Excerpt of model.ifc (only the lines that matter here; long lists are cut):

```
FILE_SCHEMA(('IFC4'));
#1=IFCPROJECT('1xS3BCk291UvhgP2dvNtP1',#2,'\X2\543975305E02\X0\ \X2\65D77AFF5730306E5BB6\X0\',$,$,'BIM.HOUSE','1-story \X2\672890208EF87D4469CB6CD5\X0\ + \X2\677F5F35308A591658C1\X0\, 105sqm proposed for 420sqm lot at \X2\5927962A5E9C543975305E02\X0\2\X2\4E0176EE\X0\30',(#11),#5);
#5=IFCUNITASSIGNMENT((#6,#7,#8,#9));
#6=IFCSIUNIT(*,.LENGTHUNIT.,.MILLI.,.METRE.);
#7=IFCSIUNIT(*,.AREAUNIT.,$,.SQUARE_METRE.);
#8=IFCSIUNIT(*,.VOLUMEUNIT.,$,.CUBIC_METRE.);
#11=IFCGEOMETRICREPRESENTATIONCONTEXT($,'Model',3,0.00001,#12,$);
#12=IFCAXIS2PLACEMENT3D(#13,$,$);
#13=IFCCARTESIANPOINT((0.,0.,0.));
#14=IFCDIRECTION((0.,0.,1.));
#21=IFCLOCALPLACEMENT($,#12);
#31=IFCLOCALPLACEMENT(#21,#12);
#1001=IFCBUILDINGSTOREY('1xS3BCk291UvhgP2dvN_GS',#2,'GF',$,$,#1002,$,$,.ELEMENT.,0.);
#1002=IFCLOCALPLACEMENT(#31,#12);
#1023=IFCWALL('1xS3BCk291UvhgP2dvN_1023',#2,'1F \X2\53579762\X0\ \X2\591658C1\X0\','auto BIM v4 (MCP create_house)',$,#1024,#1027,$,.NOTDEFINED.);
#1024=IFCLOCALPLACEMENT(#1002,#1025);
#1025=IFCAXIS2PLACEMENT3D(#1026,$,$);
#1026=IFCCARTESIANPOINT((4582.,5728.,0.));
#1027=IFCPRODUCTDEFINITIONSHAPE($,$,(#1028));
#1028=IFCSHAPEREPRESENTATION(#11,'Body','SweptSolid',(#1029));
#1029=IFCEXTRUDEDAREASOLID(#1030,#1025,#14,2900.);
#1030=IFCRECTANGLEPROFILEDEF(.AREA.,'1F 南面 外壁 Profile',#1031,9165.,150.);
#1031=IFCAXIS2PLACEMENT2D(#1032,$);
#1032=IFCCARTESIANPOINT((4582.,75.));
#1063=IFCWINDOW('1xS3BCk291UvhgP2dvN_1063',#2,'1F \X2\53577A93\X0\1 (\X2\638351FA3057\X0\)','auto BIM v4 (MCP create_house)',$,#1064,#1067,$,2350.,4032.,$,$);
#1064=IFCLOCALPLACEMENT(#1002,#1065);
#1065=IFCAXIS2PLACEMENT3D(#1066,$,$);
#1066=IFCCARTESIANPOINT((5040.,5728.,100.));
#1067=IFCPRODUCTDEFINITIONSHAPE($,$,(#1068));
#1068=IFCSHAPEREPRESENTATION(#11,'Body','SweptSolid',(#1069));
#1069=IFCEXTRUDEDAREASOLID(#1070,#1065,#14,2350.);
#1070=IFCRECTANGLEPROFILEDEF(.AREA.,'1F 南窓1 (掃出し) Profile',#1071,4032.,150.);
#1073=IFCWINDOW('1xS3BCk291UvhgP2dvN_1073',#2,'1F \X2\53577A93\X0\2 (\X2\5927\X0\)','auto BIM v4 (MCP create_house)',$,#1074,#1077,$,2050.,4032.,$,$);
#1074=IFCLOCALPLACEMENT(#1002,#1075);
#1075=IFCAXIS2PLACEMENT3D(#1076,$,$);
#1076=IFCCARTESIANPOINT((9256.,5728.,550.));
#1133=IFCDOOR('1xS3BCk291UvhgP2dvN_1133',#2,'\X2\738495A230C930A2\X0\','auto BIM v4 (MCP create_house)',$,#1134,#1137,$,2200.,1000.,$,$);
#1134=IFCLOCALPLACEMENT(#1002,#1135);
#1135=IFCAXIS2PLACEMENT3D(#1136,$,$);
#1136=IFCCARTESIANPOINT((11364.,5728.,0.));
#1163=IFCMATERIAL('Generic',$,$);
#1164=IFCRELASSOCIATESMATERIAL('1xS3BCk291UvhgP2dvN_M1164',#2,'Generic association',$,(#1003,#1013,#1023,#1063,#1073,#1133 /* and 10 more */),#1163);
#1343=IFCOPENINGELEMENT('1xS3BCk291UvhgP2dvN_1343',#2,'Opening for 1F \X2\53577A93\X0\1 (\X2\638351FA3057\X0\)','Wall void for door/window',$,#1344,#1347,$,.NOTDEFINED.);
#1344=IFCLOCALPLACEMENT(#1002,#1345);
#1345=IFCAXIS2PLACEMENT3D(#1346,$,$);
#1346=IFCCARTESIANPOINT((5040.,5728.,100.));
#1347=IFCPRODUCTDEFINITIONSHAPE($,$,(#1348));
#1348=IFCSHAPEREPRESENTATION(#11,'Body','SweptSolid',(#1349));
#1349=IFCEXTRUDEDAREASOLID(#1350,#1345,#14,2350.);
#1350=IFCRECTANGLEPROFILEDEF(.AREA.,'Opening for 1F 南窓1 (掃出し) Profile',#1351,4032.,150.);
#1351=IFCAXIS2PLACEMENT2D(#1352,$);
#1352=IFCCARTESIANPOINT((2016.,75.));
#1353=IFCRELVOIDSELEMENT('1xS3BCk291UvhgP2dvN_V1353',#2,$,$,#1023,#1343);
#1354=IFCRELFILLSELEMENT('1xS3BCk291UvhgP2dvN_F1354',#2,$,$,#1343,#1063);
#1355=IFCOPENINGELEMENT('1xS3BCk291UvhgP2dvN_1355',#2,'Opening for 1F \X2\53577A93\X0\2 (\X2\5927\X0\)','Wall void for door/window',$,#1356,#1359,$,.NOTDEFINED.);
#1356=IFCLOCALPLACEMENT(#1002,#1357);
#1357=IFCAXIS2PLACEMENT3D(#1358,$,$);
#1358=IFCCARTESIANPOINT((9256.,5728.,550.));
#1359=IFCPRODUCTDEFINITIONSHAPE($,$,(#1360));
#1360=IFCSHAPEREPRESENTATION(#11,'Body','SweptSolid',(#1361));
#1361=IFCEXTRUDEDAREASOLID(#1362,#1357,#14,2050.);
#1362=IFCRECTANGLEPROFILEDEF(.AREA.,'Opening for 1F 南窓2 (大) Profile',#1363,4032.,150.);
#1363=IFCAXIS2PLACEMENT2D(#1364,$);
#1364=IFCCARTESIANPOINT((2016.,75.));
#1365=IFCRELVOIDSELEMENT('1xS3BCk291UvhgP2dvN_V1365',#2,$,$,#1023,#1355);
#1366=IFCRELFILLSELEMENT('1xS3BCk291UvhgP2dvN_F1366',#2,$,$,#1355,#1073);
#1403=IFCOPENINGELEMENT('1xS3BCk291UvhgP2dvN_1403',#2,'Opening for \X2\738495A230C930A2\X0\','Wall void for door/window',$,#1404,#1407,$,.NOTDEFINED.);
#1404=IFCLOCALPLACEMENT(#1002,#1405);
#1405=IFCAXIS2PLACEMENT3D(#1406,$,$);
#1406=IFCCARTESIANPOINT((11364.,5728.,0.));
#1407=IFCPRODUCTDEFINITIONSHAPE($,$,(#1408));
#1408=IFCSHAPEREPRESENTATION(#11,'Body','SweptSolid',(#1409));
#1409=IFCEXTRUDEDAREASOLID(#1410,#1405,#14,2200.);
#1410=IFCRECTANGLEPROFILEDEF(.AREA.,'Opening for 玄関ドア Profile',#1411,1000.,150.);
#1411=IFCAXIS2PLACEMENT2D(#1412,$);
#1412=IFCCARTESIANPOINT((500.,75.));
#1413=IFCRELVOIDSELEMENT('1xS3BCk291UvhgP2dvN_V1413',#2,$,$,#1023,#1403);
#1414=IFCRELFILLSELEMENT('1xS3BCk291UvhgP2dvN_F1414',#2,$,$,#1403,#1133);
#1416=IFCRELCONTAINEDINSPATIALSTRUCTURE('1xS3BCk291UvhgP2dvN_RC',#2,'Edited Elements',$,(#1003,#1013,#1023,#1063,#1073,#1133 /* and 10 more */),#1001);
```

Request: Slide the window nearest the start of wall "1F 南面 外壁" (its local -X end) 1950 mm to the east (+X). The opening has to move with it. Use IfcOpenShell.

```python
import ifcopenshell
import ifcopenshell.api.geometry
import ifcopenshell.util.placement
import ifcopenshell.util.unit

model = ifcopenshell.open("model.ifc")
unit_scale = ifcopenshell.util.unit.calculate_unit_scale(model)

window = model.by_id(1063)
opening = window.FillsVoids[0].RelatingOpeningElement
wall = opening.VoidsElements[0].RelatingBuildingElement

wall_matrix = ifcopenshell.util.placement.get_local_placement(wall.ObjectPlacement)
shift = wall_matrix[:3, 0] * 1.95 / unit_scale
before = ifcopenshell.util.placement.get_local_placement(window.ObjectPlacement)[:3, 3].copy()

# The window is not placed relative to its opening, so move both.
for product in (opening, window):
    matrix = ifcopenshell.util.placement.get_local_placement(product.ObjectPlacement)
    matrix[:3, 3] += shift
    ifcopenshell.api.geometry.edit_object_placement(model, product=product, matrix=matrix, is_si=False)

after = ifcopenshell.util.placement.get_local_placement(window.ObjectPlacement)[:3, 3]
print("window moved by", (after - before).round(3) + 0.0)

model.write("model_edited.ifc")
```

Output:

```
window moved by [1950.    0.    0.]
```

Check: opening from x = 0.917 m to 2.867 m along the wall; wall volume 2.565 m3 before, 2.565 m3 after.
